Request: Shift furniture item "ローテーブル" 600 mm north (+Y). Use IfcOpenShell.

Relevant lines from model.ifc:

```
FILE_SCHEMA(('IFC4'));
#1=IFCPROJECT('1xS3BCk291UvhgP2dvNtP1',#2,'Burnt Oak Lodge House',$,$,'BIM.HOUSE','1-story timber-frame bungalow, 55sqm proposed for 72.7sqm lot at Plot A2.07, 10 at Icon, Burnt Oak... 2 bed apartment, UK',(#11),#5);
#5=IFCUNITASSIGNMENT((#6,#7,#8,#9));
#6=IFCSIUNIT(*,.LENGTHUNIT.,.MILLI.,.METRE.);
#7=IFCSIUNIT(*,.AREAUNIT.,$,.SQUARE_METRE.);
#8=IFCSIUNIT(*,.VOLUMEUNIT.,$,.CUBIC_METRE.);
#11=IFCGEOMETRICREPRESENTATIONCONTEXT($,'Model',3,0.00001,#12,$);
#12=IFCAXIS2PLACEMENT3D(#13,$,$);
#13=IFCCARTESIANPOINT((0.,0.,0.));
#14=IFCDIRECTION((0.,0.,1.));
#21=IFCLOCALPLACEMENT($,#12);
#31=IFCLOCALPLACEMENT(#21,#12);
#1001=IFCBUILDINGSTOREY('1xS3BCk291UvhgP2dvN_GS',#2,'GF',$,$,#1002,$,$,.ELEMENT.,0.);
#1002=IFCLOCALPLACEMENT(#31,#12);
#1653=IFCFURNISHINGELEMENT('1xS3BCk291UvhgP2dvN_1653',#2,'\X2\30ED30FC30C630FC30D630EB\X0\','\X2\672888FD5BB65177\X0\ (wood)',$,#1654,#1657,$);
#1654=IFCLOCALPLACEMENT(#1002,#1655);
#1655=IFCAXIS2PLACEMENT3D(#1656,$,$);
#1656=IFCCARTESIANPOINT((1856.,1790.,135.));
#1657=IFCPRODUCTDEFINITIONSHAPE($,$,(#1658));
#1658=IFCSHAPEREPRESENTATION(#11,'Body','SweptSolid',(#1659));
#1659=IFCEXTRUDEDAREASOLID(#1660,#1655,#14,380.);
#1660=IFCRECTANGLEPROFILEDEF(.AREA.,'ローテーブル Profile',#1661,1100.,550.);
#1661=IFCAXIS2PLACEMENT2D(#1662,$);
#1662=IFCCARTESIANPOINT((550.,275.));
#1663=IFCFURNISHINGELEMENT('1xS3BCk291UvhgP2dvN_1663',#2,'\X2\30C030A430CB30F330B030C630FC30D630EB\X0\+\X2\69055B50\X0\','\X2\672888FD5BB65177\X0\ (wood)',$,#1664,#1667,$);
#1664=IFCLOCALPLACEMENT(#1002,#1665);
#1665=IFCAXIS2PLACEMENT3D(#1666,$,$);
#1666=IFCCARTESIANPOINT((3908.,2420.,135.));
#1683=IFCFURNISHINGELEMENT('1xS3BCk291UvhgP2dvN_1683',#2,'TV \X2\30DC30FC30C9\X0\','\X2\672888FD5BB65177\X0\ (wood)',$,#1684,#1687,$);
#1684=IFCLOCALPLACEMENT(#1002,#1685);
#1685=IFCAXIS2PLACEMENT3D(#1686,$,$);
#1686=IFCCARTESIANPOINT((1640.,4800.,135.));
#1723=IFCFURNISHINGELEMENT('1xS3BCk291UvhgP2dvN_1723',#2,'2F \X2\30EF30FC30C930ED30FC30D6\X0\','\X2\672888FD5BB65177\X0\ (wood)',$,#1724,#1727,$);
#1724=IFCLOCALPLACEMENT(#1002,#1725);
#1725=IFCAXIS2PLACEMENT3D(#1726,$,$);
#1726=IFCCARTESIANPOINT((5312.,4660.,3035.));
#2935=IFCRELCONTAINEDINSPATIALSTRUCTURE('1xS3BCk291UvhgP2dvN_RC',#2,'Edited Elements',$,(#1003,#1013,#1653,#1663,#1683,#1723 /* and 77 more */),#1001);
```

```python
import ifcopenshell
import ifcopenshell.api.geometry
import ifcopenshell.util.placement
import ifcopenshell.util.unit

model = ifcopenshell.open("model.ifc")
unit_scale = ifcopenshell.util.unit.calculate_unit_scale(model)

item = model.by_guid("1xS3BCk291UvhgP2dvN_1653")
matrix = ifcopenshell.util.placement.get_local_placement(item.ObjectPlacement)
matrix[1, 3] += 0.6 / unit_scale
ifcopenshell.api.geometry.edit_object_placement(model, product=item, matrix=matrix, is_si=False)

print(ifcopenshell.util.placement.get_local_placement(item.ObjectPlacement).round(3) + 0.0)

model.write("model_v2.ifc")
```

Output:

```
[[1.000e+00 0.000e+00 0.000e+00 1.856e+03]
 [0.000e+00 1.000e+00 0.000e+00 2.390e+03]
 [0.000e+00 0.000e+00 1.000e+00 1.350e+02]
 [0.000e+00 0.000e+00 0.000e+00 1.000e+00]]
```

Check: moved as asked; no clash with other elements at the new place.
